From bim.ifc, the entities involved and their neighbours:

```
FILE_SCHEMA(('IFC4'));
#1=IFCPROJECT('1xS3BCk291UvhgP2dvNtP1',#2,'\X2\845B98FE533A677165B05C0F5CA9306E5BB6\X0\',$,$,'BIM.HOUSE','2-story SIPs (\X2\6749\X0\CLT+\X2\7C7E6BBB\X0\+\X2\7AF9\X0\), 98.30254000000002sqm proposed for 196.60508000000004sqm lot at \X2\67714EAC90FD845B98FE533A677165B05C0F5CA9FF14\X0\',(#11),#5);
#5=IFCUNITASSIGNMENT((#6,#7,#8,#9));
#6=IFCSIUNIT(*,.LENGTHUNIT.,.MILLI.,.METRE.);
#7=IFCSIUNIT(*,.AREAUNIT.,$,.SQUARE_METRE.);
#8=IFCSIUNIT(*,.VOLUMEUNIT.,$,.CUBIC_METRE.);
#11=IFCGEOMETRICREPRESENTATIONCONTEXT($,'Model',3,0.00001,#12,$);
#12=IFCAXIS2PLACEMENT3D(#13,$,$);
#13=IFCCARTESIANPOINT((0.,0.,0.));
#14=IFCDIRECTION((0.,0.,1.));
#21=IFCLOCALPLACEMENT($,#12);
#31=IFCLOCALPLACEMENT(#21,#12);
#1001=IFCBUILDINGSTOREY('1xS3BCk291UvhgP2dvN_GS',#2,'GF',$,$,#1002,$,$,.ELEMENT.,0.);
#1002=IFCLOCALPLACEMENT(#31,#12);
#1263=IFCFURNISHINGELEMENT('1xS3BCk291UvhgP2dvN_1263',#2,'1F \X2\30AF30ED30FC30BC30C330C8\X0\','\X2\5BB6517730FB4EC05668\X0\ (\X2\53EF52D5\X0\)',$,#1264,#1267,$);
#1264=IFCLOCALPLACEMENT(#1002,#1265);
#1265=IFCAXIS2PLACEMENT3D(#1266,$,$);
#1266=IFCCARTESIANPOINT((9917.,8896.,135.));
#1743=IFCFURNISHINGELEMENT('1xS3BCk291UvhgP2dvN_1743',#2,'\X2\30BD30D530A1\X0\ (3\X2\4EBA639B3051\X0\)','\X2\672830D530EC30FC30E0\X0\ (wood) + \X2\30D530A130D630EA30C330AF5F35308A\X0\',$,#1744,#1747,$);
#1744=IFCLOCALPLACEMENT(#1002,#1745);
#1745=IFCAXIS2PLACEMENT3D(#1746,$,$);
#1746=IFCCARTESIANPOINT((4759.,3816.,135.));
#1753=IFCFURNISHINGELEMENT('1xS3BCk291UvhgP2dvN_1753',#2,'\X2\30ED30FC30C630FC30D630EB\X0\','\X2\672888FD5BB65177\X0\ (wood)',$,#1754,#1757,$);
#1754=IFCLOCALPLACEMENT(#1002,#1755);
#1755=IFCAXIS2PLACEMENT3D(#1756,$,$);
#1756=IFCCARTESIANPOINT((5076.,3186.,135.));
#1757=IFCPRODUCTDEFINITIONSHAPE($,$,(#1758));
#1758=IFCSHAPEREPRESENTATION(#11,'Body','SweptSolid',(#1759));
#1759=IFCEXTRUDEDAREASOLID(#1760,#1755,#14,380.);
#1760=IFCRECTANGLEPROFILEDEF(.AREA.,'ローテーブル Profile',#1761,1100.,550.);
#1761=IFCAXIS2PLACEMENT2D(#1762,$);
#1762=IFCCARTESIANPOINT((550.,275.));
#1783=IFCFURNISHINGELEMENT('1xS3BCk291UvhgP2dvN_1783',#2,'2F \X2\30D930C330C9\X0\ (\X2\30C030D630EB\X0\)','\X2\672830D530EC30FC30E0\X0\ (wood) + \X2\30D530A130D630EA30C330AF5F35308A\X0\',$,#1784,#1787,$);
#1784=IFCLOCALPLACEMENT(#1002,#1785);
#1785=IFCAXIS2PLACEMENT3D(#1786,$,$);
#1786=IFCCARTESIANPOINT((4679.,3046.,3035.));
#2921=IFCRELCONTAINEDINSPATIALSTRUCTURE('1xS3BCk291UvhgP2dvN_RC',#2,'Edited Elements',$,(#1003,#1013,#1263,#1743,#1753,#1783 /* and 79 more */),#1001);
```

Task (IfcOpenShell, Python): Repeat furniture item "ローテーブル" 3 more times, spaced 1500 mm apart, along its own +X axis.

```python
import ifcopenshell
import ifcopenshell.api.geometry
import ifcopenshell.api.root
import ifcopenshell.util.element
import ifcopenshell.util.placement
import ifcopenshell.util.unit

model = ifcopenshell.open("bim.ifc")
unit_scale = ifcopenshell.util.unit.calculate_unit_scale(model)


def reuse_history(source, copy):
    """copy_class also copies each property set's owner history, people and application; keep the originals."""
    for rel in copy.IsDefinedBy:
        if rel.is_a("IfcRelDefinesByProperties") and (history := rel.RelatingPropertyDefinition.OwnerHistory):
            rel.RelatingPropertyDefinition.OwnerHistory = source.OwnerHistory
            ifcopenshell.util.element.remove_deep2(model, history)


source = model.by_guid("1xS3BCk291UvhgP2dvN_1753")
base = ifcopenshell.util.placement.get_local_placement(source.ObjectPlacement)
step = base[:3, 0] * 1.5 / unit_scale

for i in range(1, 4):
    copy = ifcopenshell.api.root.copy_class(model, product=source)
    copy.Representation = ifcopenshell.util.element.copy_deep(
        model, source.Representation, exclude=["IfcGeometricRepresentationContext", "IfcRepresentationMap"]
    )
    reuse_history(source, copy)
    matrix = base.copy()
    matrix[:3, 3] += i * step
    print("added at", matrix[:3, 3].round(3) + 0.0)
    ifcopenshell.api.geometry.edit_object_placement(model, product=copy, matrix=matrix, is_si=False)

model.write("bim-out.ifc")
```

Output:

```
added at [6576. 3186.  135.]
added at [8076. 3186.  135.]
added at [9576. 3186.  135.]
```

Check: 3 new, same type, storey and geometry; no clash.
